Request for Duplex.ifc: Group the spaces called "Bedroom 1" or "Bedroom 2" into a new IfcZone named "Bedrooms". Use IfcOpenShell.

First a look at what the model holds.

```python
import ifcopenshell

model = ifcopenshell.open("Duplex.ifc")
print(model.schema)
seen = {}
for space in model.by_type("IfcSpace"):
    seen[space.LongName] = seen.get(space.LongName, 0) + 1
for name, count in sorted(seen.items(), key=str):
    print(count, "x", name)
print("zones:", [z.Name for z in model.by_type("IfcZone")][:20])
```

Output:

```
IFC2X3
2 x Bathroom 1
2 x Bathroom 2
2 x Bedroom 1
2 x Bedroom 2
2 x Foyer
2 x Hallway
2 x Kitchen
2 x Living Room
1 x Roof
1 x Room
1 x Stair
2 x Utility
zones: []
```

```python
import ifcopenshell
import ifcopenshell.api.group
import ifcopenshell.api.root

model = ifcopenshell.open("Duplex.ifc")

names = {"Bedroom 1", "Bedroom 2"}
spaces = [s for s in model.by_type("IfcSpace") if s.LongName in names]

zone = ifcopenshell.api.root.create_entity(model, ifc_class="IfcZone", name="Bedrooms")
ifcopenshell.api.group.assign_group(model, products=spaces, group=zone)
print(len(spaces), "spaces in", zone.Name)

model.write("Duplex-out.ifc")
```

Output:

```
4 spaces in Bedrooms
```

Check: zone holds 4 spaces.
